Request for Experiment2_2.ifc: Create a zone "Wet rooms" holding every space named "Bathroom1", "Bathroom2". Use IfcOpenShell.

First a look at what the model holds.

```python
import ifcopenshell

model = ifcopenshell.open("Experiment2_2.ifc")
print(model.schema)
seen = {}
for space in model.by_type("IfcSpace"):
    seen[space.LongName] = seen.get(space.LongName, 0) + 1
for name, count in sorted(seen.items(), key=str):
    print(count, "x", name)
print("zones:", [z.Name for z in model.by_type("IfcZone")][:20])
```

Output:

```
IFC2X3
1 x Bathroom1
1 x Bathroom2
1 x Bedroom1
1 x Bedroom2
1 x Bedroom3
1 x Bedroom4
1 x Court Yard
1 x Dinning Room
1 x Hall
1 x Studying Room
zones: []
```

```python
import ifcopenshell
import ifcopenshell.api.group
import ifcopenshell.api.root

model = ifcopenshell.open("Experiment2_2.ifc")

names = {"Bathroom1", "Bathroom2"}
spaces = [s for s in model.by_type("IfcSpace") if s.LongName in names]

zone = ifcopenshell.api.root.create_entity(model, ifc_class="IfcZone", name="Wet rooms")
ifcopenshell.api.group.assign_group(model, products=spaces, group=zone)
print(len(spaces), "spaces in", zone.Name)

model.write("Experiment2_2_rev.ifc")
```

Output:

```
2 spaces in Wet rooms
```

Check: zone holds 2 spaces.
